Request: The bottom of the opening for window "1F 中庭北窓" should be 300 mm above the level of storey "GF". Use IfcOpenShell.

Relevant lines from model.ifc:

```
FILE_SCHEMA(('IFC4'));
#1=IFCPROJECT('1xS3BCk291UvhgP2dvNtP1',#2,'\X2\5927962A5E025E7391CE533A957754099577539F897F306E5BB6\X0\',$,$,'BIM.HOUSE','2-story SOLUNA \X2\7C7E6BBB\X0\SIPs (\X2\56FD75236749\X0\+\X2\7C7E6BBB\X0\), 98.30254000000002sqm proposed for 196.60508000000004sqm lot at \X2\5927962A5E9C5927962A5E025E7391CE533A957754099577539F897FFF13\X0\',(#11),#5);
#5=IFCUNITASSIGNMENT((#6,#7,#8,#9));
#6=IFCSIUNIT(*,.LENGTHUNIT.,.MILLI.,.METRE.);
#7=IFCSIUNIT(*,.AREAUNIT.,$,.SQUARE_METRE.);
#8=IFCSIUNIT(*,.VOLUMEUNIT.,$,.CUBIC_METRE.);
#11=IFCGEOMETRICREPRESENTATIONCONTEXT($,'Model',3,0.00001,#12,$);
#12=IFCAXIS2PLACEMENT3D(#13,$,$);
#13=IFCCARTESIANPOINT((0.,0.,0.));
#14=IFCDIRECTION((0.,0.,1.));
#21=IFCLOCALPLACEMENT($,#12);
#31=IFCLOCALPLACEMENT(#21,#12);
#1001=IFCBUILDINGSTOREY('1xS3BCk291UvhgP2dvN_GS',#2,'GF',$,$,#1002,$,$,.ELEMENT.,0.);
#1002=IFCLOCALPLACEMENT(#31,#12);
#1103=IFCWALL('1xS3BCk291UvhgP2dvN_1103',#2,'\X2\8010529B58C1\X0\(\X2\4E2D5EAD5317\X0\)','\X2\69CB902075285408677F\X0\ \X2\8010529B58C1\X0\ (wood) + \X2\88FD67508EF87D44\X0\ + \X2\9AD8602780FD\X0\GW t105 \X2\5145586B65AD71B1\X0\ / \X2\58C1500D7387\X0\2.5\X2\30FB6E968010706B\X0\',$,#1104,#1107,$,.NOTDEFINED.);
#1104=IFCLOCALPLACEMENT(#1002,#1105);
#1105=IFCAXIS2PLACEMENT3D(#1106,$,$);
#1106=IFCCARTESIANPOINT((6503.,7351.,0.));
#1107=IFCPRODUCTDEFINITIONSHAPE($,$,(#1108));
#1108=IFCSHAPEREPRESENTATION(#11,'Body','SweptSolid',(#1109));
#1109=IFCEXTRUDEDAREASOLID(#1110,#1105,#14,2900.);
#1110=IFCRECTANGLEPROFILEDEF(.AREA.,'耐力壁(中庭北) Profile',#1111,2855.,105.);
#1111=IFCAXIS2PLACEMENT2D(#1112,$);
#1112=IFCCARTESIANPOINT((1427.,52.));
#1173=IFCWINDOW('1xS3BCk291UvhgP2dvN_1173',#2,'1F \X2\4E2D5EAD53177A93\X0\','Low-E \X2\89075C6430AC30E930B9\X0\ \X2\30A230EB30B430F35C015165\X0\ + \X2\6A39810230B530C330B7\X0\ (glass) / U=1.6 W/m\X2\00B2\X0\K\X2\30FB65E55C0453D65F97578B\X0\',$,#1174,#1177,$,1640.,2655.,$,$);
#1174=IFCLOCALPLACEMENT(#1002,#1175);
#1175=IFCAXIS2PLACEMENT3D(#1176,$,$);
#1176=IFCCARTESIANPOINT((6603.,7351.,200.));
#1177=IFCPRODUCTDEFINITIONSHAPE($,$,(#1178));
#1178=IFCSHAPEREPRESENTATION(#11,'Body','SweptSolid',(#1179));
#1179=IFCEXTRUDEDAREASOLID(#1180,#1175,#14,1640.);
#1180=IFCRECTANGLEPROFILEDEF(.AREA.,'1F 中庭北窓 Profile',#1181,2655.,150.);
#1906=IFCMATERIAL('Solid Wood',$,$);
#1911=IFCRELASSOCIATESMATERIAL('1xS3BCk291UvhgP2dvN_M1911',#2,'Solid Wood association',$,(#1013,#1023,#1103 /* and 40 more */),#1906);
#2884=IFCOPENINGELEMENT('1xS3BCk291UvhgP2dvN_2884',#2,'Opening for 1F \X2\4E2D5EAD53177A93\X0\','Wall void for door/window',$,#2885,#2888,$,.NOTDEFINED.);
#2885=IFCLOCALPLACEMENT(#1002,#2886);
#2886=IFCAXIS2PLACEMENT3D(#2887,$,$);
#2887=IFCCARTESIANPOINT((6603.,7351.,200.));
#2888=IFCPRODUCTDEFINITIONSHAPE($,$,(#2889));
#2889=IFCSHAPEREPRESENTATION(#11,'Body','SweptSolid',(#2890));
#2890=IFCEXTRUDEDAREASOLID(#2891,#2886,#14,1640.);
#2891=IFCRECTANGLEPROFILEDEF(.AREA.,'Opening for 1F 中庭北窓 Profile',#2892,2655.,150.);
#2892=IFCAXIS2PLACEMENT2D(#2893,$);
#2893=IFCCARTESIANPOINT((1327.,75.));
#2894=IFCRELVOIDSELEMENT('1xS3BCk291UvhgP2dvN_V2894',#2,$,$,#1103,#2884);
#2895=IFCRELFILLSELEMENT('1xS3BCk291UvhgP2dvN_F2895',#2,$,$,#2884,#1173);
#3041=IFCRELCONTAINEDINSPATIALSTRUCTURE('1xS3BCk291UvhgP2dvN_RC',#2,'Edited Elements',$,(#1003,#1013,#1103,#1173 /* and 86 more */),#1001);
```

```python
import numpy as np
import ifcopenshell
import ifcopenshell.api.geometry
import ifcopenshell.geom
import ifcopenshell.util.element
import ifcopenshell.util.placement
import ifcopenshell.util.shape
import ifcopenshell.util.unit

model = ifcopenshell.open("model.ifc")
unit_scale = ifcopenshell.util.unit.calculate_unit_scale(model)

window = model.by_guid("1xS3BCk291UvhgP2dvN_1173")
opening = window.FillsVoids[0].RelatingOpeningElement
storey = ifcopenshell.util.element.get_container(window, ifc_class="IfcBuildingStorey")
level = ifcopenshell.util.placement.get_local_placement(storey.ObjectPlacement)[2, 3]

# The opening's origin need not be at the sill, so measure its lowest point.
shape = ifcopenshell.geom.create_shape(ifcopenshell.geom.settings(), opening)
bottom = ifcopenshell.util.shape.get_shape_bottom_elevation(shape, shape.geometry) / unit_scale
dz = level + 300.0 - bottom

shift = np.array([0.0, 0.0, dz])
# The window is not placed relative to its opening, so move both.
for product in (opening, window):
    matrix = ifcopenshell.util.placement.get_local_placement(product.ObjectPlacement)
    matrix[:3, 3] += shift
    ifcopenshell.api.geometry.edit_object_placement(model, product=product, matrix=matrix, is_si=False)

print(f"moved by {dz * unit_scale:+.3f} m")

model.write("model_edited.ifc")
```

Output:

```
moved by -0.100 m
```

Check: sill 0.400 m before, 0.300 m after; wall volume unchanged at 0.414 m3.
